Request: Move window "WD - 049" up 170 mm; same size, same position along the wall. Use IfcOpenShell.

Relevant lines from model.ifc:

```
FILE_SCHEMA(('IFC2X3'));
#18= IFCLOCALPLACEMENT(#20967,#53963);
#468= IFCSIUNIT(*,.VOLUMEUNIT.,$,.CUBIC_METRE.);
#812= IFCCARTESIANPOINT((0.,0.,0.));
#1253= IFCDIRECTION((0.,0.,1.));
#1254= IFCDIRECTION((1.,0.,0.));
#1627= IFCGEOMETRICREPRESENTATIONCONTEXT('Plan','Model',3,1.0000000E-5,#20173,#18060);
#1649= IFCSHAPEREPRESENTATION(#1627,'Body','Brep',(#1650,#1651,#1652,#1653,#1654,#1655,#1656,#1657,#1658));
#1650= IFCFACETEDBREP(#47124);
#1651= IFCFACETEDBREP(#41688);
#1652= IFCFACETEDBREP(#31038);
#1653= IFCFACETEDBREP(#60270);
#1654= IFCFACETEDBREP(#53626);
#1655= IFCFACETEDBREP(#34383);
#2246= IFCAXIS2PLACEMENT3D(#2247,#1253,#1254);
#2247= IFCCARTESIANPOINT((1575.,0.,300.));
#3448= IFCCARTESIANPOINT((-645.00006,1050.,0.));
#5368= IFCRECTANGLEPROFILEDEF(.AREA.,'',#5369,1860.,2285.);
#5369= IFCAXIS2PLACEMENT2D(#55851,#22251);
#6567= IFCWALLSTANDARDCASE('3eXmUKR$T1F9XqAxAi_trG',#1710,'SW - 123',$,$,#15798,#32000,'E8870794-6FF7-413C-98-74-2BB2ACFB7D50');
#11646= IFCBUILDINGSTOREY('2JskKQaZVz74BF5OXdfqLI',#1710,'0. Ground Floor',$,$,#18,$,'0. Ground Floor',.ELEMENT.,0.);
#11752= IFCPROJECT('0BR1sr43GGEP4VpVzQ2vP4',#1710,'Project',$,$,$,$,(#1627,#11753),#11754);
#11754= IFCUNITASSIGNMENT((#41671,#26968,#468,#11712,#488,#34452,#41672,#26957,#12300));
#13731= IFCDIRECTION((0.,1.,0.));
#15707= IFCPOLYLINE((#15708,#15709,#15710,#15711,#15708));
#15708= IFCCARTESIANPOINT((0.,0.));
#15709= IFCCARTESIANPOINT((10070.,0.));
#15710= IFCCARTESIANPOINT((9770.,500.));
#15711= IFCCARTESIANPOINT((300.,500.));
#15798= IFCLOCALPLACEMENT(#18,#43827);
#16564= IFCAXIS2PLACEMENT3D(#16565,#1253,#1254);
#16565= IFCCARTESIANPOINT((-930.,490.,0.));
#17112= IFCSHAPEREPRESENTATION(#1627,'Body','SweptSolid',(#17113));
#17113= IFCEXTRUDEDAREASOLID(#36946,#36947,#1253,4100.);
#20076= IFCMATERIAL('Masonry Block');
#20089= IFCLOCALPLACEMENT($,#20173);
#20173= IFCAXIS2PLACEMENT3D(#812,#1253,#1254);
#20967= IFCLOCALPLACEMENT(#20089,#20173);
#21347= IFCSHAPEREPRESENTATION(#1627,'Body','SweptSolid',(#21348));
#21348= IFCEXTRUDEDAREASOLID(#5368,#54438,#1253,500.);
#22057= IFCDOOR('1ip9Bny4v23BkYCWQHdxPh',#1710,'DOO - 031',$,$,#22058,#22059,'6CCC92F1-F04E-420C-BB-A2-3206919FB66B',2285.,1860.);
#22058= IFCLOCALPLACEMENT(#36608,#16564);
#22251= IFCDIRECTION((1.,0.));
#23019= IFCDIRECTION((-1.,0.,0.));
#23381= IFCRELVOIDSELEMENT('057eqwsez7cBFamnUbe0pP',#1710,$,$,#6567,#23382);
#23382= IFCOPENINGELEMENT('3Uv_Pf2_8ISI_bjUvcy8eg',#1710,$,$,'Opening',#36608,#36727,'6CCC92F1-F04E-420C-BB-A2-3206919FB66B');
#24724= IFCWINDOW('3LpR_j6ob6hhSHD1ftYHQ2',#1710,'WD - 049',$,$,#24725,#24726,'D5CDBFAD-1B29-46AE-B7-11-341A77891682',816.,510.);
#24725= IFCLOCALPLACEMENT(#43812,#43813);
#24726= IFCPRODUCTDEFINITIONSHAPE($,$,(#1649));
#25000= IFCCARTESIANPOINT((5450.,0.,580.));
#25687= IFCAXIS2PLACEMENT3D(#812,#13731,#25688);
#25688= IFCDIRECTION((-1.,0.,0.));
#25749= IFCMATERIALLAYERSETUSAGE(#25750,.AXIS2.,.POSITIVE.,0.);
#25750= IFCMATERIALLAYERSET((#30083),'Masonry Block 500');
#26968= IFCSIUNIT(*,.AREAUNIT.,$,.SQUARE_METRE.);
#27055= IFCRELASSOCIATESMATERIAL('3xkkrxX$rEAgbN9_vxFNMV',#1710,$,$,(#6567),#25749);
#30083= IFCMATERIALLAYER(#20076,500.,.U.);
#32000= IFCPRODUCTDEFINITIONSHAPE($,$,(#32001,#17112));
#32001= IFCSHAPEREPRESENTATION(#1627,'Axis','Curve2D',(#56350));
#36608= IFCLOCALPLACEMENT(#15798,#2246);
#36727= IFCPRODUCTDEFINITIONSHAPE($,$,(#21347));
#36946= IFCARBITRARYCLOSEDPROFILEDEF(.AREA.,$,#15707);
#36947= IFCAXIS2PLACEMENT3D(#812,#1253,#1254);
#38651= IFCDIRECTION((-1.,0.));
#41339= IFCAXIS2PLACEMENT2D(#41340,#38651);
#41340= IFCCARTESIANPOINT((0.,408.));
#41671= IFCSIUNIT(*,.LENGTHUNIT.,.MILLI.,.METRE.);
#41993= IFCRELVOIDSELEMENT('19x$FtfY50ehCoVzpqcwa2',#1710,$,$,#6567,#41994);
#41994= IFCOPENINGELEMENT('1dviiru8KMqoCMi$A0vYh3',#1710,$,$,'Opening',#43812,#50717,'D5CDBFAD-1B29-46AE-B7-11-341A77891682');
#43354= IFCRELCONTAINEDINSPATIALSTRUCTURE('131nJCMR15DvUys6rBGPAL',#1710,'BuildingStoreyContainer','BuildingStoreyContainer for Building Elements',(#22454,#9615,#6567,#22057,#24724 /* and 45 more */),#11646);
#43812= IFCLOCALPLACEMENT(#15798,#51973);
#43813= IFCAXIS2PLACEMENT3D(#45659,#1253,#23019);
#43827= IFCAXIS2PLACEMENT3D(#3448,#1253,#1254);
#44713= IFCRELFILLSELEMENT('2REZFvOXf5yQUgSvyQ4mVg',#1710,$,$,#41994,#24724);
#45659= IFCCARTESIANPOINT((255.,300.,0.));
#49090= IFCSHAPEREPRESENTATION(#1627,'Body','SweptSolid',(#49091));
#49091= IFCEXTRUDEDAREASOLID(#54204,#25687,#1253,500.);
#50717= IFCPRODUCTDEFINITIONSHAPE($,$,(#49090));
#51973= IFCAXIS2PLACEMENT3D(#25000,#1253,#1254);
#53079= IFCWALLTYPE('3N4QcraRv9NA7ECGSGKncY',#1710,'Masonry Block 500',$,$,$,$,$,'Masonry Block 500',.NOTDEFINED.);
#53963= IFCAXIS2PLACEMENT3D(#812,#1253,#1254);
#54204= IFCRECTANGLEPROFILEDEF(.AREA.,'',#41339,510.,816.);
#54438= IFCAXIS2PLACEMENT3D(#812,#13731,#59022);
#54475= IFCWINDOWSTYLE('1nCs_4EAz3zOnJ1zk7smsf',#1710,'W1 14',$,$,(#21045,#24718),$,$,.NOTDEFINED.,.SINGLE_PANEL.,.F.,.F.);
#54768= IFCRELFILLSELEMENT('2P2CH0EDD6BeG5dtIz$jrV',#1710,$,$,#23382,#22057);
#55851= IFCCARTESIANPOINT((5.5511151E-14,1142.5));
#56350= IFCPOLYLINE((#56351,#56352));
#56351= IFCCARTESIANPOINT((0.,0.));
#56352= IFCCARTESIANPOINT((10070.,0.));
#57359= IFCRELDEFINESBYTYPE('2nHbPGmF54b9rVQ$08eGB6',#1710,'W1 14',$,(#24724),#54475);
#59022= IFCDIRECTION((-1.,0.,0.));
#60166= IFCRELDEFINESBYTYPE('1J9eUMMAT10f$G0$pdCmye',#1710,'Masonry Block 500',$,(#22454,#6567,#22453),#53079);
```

```python
import numpy as np
import ifcopenshell
import ifcopenshell.api.geometry
import ifcopenshell.util.placement
import ifcopenshell.util.unit

model = ifcopenshell.open("model.ifc")
unit_scale = ifcopenshell.util.unit.calculate_unit_scale(model)

window = model.by_guid("3LpR_j6ob6hhSHD1ftYHQ2")
opening = window.FillsVoids[0].RelatingOpeningElement
dz = 170.0

shift = np.array([0.0, 0.0, dz])
# The window is placed relative to its opening, so it follows when the opening moves.
matrix = ifcopenshell.util.placement.get_local_placement(opening.ObjectPlacement)
matrix[:3, 3] += shift
ifcopenshell.api.geometry.edit_object_placement(
    model, product=opening, matrix=matrix, is_si=False, should_transform_children=True
)

print(f"moved by {dz * unit_scale:+.3f} m")

model.write("model-out.ifc")
```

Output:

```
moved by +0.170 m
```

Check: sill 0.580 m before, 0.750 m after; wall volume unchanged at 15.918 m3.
